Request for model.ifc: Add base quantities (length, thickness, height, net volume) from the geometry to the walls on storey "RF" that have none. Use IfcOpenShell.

First a look at what the model holds.

```python
import ifcopenshell
import ifcopenshell.util.element
import ifcopenshell.util.unit

model = ifcopenshell.open("model.ifc")
print(model.schema)
for unit_type in ("LENGTHUNIT", "AREAUNIT", "VOLUMEUNIT"):
    print(unit_type, ifcopenshell.util.unit.calculate_unit_scale(model, unit_type))
storey = next(s for s in model.by_type("IfcBuildingStorey") if s.Name == "RF")
walls = [e for e in ifcopenshell.util.element.get_decomposition(storey) if e.is_a("IfcWall")]
for e in sorted(walls, key=lambda e: e.id()):
    print(e.id(), e.is_a(), e.Name, list(ifcopenshell.util.element.get_psets(e, qtos_only=True)), sep=" | ")
```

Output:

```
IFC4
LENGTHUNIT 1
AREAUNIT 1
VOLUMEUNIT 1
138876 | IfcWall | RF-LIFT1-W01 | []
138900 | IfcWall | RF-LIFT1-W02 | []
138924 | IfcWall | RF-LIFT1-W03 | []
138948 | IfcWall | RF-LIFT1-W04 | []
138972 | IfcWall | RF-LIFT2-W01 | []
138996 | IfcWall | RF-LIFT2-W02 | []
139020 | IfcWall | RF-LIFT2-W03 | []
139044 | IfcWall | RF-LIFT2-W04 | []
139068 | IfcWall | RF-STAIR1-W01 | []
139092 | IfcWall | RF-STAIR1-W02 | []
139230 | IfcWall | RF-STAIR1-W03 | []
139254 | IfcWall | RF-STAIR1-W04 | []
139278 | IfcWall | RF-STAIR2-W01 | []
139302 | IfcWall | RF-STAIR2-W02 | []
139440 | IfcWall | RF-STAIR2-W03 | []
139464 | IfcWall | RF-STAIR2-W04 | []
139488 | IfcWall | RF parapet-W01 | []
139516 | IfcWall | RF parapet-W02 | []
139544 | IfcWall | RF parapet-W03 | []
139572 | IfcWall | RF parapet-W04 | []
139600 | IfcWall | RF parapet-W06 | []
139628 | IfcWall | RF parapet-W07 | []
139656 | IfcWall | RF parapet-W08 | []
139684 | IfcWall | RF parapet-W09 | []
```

```python
import ifcopenshell
import ifcopenshell.api.pset
import ifcopenshell.geom
import ifcopenshell.util.element
import ifcopenshell.util.shape
import ifcopenshell.util.unit

model = ifcopenshell.open("model.ifc")
unit_scale = ifcopenshell.util.unit.calculate_unit_scale(model)
volume_scale = ifcopenshell.util.unit.calculate_unit_scale(model, "VOLUMEUNIT")
settings = ifcopenshell.geom.settings()

storey = next(s for s in model.by_type("IfcBuildingStorey") if s.Name == "RF")
walls = [e for e in ifcopenshell.util.element.get_decomposition(storey) if e.is_a("IfcWall")]

for e in sorted(walls, key=lambda e: e.id()):
    if ifcopenshell.util.element.get_psets(e, qtos_only=True, should_inherit=False):
        continue
    # Geometry comes back in metres, in the element's own axes.
    shape = ifcopenshell.geom.create_shape(settings, e)
    values = {
        "Length": ifcopenshell.util.shape.get_x(shape.geometry) / unit_scale,
        "Width": ifcopenshell.util.shape.get_y(shape.geometry) / unit_scale,
        "Height": ifcopenshell.util.shape.get_z(shape.geometry) / unit_scale,
        "NetVolume": ifcopenshell.util.shape.get_volume(shape.geometry) / volume_scale,
    }
    qto = ifcopenshell.api.pset.add_qto(model, product=e, name="Qto_WallBaseQuantities")
    ifcopenshell.api.pset.edit_qto(model, qto=qto, properties=values)
    print(e.id(), {k: round(v, 3) for k, v in values.items()})

model.write("model_v2.ifc")
```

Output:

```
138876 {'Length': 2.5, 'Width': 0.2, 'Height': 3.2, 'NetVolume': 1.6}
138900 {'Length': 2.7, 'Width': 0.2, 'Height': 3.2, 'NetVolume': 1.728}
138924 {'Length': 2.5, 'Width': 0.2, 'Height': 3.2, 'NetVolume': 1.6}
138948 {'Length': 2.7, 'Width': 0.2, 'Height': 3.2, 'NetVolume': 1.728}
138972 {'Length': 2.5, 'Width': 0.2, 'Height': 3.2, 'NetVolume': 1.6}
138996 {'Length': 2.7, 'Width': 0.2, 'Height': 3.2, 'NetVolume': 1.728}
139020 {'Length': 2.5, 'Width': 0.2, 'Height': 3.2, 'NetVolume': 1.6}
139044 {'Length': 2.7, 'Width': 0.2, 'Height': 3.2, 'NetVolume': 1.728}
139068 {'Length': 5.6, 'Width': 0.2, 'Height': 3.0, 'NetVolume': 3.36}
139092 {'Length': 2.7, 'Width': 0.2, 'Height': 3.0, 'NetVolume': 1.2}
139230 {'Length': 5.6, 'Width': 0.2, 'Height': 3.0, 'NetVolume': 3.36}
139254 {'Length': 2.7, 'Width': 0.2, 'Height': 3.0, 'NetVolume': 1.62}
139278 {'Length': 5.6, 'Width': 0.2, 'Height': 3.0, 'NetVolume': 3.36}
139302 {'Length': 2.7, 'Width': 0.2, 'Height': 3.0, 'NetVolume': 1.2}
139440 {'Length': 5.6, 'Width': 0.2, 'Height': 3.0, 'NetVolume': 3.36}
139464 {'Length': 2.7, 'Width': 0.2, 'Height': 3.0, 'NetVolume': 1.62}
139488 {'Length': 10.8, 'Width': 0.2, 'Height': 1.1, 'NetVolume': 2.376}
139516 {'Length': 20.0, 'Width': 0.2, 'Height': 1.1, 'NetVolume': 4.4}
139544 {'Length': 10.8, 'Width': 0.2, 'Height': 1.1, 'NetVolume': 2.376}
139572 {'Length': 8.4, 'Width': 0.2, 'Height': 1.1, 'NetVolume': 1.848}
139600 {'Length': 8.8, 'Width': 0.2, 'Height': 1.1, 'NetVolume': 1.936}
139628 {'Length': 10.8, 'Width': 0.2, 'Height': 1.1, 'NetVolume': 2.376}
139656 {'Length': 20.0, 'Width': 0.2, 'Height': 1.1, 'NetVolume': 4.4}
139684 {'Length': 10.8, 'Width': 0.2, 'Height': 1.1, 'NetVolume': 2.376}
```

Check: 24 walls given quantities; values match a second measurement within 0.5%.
